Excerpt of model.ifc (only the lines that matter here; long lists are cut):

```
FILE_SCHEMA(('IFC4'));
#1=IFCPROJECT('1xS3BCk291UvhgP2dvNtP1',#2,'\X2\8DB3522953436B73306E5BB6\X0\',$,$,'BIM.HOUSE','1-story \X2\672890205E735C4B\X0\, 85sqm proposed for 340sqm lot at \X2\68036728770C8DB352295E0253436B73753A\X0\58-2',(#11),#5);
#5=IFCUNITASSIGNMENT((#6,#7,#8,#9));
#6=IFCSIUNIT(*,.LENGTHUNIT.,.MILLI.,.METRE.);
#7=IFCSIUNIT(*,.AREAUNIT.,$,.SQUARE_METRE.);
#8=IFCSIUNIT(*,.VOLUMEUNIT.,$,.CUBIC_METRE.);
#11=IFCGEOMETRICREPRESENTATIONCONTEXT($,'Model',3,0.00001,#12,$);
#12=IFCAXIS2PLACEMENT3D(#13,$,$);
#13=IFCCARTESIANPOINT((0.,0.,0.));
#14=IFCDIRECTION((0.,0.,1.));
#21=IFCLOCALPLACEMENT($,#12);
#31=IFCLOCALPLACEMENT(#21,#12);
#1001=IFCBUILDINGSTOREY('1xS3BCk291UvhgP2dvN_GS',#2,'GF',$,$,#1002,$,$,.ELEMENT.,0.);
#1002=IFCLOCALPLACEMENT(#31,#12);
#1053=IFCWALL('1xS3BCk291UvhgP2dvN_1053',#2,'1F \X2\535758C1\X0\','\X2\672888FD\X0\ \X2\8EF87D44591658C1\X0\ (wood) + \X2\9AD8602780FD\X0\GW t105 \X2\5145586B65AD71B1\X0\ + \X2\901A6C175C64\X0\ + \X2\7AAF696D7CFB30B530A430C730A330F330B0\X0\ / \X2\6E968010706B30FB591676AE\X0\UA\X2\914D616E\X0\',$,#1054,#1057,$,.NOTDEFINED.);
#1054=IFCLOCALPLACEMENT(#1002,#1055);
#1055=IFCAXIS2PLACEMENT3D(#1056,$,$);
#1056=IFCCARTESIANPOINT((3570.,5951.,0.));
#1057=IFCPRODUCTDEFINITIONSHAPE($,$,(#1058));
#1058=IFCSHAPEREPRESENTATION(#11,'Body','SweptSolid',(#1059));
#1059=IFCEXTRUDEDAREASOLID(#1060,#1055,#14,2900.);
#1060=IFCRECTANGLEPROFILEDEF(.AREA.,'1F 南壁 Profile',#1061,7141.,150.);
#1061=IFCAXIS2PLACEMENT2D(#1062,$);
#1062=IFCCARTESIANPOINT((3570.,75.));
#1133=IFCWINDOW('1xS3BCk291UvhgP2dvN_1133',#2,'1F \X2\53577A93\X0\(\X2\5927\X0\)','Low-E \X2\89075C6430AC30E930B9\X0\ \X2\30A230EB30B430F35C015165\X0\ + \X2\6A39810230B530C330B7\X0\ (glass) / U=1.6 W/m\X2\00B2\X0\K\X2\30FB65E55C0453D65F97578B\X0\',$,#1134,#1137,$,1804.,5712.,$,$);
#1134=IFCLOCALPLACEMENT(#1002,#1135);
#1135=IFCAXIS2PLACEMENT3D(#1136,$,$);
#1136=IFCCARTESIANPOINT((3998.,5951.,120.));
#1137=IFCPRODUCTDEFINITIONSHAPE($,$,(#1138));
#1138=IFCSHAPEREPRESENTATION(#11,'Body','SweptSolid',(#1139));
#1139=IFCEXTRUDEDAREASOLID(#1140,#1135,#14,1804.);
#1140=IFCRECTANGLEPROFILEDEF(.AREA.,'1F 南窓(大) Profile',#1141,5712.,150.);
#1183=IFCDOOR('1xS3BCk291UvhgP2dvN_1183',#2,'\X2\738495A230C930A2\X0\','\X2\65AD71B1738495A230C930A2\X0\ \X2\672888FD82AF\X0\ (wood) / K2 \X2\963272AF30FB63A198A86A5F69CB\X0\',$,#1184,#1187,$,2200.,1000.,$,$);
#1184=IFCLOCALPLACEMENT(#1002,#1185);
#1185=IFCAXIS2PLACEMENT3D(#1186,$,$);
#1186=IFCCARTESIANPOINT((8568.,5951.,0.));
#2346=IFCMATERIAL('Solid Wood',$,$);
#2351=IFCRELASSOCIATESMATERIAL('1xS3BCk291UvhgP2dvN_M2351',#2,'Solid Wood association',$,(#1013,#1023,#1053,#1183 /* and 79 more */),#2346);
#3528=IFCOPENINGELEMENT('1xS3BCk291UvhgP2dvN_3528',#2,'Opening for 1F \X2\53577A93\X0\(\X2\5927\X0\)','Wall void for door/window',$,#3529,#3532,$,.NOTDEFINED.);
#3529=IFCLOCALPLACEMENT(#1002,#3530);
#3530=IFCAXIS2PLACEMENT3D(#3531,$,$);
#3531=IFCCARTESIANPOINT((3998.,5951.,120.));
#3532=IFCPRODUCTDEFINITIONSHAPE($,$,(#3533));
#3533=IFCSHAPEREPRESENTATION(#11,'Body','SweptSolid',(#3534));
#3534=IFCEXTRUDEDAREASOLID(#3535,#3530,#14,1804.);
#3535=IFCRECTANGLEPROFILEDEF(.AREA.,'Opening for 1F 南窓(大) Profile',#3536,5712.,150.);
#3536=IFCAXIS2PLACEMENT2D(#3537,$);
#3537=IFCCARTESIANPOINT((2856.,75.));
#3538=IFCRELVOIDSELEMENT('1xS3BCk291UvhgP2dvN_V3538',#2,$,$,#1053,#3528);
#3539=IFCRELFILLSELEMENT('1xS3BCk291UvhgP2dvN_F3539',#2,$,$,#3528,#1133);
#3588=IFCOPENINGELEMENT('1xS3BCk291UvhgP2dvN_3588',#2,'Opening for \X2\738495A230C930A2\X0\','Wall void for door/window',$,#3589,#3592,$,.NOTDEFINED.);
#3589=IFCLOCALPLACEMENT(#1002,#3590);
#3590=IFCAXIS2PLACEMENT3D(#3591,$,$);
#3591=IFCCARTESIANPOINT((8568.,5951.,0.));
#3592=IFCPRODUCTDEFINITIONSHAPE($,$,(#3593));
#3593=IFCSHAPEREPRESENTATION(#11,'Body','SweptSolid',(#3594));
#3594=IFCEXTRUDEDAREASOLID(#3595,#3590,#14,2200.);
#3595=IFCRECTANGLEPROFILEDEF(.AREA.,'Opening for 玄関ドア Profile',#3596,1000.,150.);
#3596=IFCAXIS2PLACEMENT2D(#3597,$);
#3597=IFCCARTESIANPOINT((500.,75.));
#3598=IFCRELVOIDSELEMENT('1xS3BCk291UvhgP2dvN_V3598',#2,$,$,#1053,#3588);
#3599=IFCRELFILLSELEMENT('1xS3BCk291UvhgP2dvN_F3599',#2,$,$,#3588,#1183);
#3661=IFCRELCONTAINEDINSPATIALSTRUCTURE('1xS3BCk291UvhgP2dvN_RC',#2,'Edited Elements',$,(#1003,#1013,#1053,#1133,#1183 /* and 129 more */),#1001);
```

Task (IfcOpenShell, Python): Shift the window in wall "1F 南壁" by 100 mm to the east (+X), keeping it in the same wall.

```python
import ifcopenshell
import ifcopenshell.api.geometry
import ifcopenshell.util.placement

model = ifcopenshell.open("model.ifc")

window = model.by_guid("1xS3BCk291UvhgP2dvN_1133")
opening = window.FillsVoids[0].RelatingOpeningElement
wall = opening.VoidsElements[0].RelatingBuildingElement

wall_matrix = ifcopenshell.util.placement.get_local_placement(wall.ObjectPlacement)
shift = wall_matrix[:3, 0] * 100.0
before = ifcopenshell.util.placement.get_local_placement(window.ObjectPlacement)[:3, 3].copy()

# The window is not placed relative to its opening, so move both.
for product in (opening, window):
    matrix = ifcopenshell.util.placement.get_local_placement(product.ObjectPlacement)
    matrix[:3, 3] += shift
    ifcopenshell.api.geometry.edit_object_placement(model, product=product, matrix=matrix, is_si=False)

after = ifcopenshell.util.placement.get_local_placement(window.ObjectPlacement)[:3, 3]
print("window moved by", (after - before).round(3) + 0.0)

model.write("model_rev.ifc")
```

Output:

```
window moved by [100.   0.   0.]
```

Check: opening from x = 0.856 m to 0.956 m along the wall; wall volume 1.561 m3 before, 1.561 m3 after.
